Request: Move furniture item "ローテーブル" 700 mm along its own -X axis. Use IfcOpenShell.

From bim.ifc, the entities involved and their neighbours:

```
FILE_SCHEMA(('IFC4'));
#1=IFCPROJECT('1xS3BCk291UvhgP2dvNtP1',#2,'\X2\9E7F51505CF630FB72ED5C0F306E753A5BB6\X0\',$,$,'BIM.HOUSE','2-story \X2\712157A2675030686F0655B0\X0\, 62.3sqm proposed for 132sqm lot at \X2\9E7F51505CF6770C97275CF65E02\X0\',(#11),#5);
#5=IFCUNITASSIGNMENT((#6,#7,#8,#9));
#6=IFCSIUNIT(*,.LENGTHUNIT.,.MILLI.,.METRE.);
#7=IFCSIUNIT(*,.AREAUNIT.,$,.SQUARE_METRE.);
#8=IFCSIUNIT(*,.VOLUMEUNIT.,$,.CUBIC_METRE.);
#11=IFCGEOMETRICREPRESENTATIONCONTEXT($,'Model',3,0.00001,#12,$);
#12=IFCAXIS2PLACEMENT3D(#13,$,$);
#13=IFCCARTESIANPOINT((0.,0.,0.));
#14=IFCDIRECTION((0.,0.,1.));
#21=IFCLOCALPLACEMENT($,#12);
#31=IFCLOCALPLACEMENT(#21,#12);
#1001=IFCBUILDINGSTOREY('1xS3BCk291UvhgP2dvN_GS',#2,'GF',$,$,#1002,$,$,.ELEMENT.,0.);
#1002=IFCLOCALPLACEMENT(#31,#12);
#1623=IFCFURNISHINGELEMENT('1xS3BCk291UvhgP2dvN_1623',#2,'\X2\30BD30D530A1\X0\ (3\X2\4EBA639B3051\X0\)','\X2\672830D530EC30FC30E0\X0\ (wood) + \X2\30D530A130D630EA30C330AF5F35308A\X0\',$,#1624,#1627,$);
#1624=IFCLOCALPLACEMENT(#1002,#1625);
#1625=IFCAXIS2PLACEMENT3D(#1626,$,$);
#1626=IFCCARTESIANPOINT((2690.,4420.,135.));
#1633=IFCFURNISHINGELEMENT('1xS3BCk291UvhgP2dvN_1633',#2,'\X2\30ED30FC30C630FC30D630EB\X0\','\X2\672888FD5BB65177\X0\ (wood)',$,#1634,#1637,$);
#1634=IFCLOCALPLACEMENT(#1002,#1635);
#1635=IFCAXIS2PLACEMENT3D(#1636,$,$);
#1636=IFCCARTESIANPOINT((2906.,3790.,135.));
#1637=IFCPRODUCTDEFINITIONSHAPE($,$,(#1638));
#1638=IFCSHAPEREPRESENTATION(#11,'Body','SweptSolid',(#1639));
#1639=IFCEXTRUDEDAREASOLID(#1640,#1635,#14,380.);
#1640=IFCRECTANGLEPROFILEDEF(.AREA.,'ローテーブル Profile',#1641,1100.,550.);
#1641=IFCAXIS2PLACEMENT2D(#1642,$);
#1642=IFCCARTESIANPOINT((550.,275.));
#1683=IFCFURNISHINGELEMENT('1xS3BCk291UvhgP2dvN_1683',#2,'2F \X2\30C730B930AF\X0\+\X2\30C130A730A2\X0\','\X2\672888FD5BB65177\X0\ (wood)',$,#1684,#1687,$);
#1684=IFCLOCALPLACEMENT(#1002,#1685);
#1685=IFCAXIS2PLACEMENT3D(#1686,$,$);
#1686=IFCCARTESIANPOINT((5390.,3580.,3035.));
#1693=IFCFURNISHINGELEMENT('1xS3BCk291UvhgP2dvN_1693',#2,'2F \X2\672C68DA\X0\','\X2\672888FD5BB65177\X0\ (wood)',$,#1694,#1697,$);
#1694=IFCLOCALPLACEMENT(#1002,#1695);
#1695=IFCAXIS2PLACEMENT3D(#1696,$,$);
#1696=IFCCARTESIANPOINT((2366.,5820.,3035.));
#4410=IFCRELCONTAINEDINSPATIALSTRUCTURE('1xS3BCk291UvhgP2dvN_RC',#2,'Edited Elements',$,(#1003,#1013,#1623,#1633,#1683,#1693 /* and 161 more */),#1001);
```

```python
import ifcopenshell
import ifcopenshell.api.geometry
import ifcopenshell.util.placement
import ifcopenshell.util.unit

model = ifcopenshell.open("bim.ifc")
unit_scale = ifcopenshell.util.unit.calculate_unit_scale(model)

item = model.by_guid("1xS3BCk291UvhgP2dvN_1633")
matrix = ifcopenshell.util.placement.get_local_placement(item.ObjectPlacement)
matrix[:3, 3] -= matrix[:3, 0] * 0.7 / unit_scale
ifcopenshell.api.geometry.edit_object_placement(model, product=item, matrix=matrix, is_si=False)

print(ifcopenshell.util.placement.get_local_placement(item.ObjectPlacement).round(3) + 0.0)

model.write("bim_rev.ifc")
```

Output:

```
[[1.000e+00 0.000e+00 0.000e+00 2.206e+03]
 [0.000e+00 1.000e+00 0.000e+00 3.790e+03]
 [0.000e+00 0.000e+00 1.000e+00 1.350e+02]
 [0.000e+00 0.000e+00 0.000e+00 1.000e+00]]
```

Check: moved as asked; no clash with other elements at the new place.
